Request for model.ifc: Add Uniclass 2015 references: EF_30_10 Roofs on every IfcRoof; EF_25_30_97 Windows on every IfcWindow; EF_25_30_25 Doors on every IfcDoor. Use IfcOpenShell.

First a look at what the model holds.

```python
import ifcopenshell

model = ifcopenshell.open("model.ifc")
print(model.schema)
print("classifications:", [c.Name for c in model.by_type("IfcClassification")])
for ifc_class in ("IfcDoor", "IfcRoof", "IfcStair", "IfcWall", "IfcWindow"):
    print(ifc_class, len(model.by_type(ifc_class)))
```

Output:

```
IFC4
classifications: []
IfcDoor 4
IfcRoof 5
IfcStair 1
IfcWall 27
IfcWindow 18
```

```python
import ifcopenshell
import ifcopenshell.api.classification

model = ifcopenshell.open("model.ifc")

system = ifcopenshell.api.classification.add_classification(model, classification="Uniclass 2015")

codes = {
    "IfcRoof": ("EF_30_10", "Roofs"),
    "IfcWindow": ("EF_25_30_97", "Windows"),
    "IfcDoor": ("EF_25_30_25", "Doors"),
}
for ifc_class, (code, name) in codes.items():
    products = model.by_type(ifc_class)
    ifcopenshell.api.classification.add_reference(
        model, products=products, classification=system, identification=code, name=name
    )
    print(code, len(products))

model.write("model_v2.ifc")
```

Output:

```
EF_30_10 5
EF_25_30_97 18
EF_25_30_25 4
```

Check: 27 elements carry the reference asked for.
